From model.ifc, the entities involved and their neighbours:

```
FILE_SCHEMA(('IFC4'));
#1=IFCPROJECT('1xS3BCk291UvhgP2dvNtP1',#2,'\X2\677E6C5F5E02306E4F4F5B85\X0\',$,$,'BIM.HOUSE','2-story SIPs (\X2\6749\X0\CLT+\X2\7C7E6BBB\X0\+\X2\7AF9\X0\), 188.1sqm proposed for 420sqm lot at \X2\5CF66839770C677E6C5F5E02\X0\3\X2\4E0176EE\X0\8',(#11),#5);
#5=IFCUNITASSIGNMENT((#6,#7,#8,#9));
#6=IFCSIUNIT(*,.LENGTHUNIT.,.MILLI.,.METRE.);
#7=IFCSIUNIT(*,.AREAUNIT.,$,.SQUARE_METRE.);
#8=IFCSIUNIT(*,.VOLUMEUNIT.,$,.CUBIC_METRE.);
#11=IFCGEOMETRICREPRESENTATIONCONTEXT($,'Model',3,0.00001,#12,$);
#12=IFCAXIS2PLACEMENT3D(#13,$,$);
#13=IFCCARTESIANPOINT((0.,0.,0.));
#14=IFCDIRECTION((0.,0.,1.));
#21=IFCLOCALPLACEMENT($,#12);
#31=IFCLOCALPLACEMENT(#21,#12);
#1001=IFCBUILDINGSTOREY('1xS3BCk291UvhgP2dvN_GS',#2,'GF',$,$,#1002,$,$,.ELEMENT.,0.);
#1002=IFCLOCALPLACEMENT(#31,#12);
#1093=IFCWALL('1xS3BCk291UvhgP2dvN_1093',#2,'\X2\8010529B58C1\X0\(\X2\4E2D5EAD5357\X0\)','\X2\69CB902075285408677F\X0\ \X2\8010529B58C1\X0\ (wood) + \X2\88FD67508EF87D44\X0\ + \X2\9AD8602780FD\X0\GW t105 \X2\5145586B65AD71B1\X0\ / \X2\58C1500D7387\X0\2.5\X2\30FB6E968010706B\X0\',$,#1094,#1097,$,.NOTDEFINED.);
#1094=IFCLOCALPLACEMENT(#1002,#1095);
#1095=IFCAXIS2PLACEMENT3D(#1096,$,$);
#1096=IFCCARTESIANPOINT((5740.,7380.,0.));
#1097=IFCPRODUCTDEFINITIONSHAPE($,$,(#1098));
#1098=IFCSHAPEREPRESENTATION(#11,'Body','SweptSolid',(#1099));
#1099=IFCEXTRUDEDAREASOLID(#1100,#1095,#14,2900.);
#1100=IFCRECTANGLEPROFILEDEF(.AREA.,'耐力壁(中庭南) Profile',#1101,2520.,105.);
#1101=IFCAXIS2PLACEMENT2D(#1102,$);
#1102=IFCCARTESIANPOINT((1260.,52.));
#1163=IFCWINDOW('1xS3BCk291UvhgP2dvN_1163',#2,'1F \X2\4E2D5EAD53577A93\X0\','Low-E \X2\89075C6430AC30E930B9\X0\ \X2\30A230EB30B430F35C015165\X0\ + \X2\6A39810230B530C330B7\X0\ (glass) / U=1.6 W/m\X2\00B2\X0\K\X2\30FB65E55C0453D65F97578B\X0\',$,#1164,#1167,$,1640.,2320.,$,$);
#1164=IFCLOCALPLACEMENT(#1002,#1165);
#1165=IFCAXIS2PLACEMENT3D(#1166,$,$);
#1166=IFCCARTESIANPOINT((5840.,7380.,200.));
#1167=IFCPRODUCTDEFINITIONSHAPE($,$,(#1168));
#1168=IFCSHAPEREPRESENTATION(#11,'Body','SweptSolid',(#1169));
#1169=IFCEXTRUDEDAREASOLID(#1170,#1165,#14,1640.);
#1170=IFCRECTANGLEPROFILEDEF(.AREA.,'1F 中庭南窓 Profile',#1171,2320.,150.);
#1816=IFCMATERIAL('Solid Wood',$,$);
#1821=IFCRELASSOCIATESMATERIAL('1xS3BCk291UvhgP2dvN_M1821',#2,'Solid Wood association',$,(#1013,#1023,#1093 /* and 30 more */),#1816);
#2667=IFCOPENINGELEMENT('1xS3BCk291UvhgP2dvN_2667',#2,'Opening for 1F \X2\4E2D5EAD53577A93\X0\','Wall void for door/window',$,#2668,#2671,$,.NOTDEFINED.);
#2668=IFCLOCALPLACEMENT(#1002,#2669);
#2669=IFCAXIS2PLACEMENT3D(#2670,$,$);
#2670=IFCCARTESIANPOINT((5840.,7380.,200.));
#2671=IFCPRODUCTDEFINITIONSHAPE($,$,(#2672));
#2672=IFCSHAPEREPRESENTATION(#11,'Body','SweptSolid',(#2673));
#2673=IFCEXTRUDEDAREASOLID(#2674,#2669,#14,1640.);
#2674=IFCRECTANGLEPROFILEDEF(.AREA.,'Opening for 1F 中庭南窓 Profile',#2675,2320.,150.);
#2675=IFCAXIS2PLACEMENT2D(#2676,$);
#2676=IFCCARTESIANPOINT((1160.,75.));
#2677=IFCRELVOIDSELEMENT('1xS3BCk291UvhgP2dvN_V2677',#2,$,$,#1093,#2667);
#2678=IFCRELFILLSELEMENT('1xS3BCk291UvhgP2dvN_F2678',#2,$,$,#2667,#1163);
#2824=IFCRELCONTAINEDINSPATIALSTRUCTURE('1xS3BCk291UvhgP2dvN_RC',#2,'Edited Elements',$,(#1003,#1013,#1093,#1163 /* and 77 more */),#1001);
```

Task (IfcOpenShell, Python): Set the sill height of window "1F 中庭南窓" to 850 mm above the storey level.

```python
import numpy as np
import ifcopenshell
import ifcopenshell.api.geometry
import ifcopenshell.geom
import ifcopenshell.util.element
import ifcopenshell.util.placement
import ifcopenshell.util.shape
import ifcopenshell.util.unit

model = ifcopenshell.open("model.ifc")
unit_scale = ifcopenshell.util.unit.calculate_unit_scale(model)

window = model.by_id(1163)
opening = window.FillsVoids[0].RelatingOpeningElement
storey = ifcopenshell.util.element.get_container(window, ifc_class="IfcBuildingStorey")
level = ifcopenshell.util.placement.get_local_placement(storey.ObjectPlacement)[2, 3]

# The opening's origin need not be at the sill, so measure its lowest point.
shape = ifcopenshell.geom.create_shape(ifcopenshell.geom.settings(), opening)
bottom = ifcopenshell.util.shape.get_shape_bottom_elevation(shape, shape.geometry) / unit_scale
dz = level + 850.0 - bottom

shift = np.array([0.0, 0.0, dz])
# The window is not placed relative to its opening, so move both.
for product in (opening, window):
    matrix = ifcopenshell.util.placement.get_local_placement(product.ObjectPlacement)
    matrix[:3, 3] += shift
    ifcopenshell.api.geometry.edit_object_placement(model, product=product, matrix=matrix, is_si=False)

print(f"moved by {dz * unit_scale:+.3f} m")

model.write("model_updated.ifc")
```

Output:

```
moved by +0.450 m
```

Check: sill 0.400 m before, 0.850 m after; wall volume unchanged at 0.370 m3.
